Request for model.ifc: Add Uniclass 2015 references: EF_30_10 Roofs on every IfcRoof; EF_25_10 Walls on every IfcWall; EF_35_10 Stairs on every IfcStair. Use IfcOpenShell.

First a look at what the model holds.

```python
import ifcopenshell

model = ifcopenshell.open("model.ifc")
print(model.schema)
print("classifications:", [c.Name for c in model.by_type("IfcClassification")])
for ifc_class in ("IfcDoor", "IfcRoof", "IfcStair", "IfcWall", "IfcWindow"):
    print(ifc_class, len(model.by_type(ifc_class)))
```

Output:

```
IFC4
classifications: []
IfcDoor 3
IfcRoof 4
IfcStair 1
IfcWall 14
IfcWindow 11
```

```python
import ifcopenshell
import ifcopenshell.api.classification

model = ifcopenshell.open("model.ifc")

system = ifcopenshell.api.classification.add_classification(model, classification="Uniclass 2015")

codes = {
    "IfcRoof": ("EF_30_10", "Roofs"),
    "IfcWall": ("EF_25_10", "Walls"),
    "IfcStair": ("EF_35_10", "Stairs"),
}
for ifc_class, (code, name) in codes.items():
    products = model.by_type(ifc_class)
    ifcopenshell.api.classification.add_reference(
        model, products=products, classification=system, identification=code, name=name
    )
    print(code, len(products))

model.write("model-out.ifc")
```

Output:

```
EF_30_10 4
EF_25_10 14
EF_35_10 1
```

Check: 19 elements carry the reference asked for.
